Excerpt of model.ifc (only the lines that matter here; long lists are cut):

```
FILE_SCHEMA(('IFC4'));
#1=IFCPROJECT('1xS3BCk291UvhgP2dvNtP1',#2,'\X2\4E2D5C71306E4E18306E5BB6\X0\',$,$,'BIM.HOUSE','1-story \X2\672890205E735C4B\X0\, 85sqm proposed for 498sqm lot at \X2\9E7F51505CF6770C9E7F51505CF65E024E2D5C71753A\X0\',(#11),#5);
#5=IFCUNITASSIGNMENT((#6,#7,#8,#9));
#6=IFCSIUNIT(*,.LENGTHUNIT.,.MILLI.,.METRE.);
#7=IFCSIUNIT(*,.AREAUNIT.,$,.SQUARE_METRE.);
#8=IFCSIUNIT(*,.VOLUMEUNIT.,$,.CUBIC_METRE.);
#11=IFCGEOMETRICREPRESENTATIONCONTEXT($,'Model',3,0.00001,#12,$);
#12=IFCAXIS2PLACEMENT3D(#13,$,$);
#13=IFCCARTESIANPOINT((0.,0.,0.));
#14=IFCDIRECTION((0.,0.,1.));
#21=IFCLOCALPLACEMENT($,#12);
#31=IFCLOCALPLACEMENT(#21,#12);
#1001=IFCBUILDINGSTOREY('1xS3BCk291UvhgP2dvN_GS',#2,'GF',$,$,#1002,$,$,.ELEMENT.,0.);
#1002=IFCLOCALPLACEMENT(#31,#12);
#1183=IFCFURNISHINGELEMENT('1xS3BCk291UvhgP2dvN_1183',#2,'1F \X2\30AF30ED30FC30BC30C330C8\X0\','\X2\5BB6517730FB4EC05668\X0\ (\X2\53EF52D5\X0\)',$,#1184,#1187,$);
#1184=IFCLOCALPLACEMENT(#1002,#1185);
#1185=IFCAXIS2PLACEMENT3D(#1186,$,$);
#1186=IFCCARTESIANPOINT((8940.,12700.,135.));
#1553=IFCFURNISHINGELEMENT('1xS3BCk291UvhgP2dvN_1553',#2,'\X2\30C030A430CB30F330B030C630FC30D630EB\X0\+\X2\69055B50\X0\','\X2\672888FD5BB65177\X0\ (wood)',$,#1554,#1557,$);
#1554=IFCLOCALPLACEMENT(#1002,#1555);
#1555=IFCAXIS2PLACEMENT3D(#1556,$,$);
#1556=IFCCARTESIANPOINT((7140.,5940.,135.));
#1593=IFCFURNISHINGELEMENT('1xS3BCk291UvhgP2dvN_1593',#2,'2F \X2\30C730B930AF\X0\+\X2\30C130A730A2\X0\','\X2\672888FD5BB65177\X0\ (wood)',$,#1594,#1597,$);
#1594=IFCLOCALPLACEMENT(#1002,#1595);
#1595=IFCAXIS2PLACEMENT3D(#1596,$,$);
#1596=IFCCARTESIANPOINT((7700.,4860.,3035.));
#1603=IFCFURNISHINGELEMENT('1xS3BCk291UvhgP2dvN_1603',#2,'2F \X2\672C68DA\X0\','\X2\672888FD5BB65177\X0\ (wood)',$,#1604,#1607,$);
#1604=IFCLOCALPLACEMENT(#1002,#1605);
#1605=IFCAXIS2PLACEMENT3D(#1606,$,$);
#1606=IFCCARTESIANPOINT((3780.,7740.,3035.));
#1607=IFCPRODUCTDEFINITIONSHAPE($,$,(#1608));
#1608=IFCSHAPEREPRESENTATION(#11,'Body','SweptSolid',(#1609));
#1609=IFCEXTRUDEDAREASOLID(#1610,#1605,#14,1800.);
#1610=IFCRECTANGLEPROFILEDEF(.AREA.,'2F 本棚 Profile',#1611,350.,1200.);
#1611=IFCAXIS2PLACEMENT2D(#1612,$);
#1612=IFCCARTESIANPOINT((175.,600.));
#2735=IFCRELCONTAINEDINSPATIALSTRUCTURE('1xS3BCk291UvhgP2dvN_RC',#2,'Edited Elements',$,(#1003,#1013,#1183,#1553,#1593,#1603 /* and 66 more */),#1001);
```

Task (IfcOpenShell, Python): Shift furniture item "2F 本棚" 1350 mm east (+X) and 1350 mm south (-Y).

```python
import ifcopenshell
import ifcopenshell.api.geometry
import ifcopenshell.util.placement

model = ifcopenshell.open("model.ifc")

item = model.by_guid("1xS3BCk291UvhgP2dvN_1603")
matrix = ifcopenshell.util.placement.get_local_placement(item.ObjectPlacement)
matrix[0, 3] += 1350.0
matrix[1, 3] -= 1350.0
ifcopenshell.api.geometry.edit_object_placement(model, product=item, matrix=matrix, is_si=False)

print(ifcopenshell.util.placement.get_local_placement(item.ObjectPlacement).round(3) + 0.0)

model.write("model_updated.ifc")
```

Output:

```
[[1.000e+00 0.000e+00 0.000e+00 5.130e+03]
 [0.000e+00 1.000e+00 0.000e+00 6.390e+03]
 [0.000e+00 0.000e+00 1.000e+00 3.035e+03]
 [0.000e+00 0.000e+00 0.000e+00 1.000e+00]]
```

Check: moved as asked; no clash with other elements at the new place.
